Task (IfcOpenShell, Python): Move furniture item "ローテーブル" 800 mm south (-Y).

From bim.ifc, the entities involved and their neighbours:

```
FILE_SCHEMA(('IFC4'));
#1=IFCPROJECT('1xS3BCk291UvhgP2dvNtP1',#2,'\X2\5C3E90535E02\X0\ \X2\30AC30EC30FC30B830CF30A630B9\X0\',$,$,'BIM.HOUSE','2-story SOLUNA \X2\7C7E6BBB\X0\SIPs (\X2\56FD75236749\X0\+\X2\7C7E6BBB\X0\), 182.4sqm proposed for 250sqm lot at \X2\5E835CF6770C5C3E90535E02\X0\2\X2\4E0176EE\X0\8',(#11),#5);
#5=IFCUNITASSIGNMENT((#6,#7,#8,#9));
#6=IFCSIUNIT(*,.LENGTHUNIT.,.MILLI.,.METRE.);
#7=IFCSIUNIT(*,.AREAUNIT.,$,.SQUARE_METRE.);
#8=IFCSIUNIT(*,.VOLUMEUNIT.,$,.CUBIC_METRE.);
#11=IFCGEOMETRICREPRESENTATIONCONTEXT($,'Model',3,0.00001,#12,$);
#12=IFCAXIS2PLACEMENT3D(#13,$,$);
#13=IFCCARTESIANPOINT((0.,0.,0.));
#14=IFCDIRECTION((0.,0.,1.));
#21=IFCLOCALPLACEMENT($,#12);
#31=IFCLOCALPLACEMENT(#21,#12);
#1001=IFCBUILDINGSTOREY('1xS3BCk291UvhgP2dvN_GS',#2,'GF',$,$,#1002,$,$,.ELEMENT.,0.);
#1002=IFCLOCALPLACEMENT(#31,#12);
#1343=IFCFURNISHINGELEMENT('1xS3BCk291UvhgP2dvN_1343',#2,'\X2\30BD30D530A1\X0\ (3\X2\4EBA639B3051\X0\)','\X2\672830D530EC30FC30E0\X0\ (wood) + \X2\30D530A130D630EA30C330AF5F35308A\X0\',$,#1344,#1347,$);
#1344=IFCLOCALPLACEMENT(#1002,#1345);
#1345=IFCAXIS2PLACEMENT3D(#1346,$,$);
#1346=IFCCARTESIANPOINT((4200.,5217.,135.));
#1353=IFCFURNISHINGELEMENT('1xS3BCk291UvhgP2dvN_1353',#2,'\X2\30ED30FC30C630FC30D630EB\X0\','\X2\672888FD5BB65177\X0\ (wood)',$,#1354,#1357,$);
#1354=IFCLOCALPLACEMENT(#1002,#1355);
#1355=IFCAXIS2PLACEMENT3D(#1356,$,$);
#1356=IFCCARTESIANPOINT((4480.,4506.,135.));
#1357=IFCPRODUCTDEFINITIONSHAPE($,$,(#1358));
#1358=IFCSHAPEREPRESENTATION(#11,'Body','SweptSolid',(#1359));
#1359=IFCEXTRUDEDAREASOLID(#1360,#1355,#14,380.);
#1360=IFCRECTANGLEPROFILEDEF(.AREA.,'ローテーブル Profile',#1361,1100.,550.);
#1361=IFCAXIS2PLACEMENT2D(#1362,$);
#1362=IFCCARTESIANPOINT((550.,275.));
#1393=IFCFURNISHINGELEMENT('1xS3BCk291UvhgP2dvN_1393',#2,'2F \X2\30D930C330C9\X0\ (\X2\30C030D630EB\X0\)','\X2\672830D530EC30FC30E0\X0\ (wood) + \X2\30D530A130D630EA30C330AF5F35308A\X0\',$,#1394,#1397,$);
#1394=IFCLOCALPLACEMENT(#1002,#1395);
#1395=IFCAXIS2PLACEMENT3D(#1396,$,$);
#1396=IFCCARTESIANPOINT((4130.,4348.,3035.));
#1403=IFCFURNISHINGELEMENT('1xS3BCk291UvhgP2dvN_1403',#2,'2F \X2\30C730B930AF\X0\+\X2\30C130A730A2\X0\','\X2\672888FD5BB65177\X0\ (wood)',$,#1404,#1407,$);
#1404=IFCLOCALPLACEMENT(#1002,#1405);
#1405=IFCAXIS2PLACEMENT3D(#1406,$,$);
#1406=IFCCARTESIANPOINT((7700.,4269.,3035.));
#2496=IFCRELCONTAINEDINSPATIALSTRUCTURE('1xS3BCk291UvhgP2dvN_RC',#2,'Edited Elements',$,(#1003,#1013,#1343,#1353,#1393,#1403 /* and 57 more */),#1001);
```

```python
import ifcopenshell
import ifcopenshell.api.geometry
import ifcopenshell.util.placement

model = ifcopenshell.open("bim.ifc")

item = model.by_id(1353)
matrix = ifcopenshell.util.placement.get_local_placement(item.ObjectPlacement)
matrix[1, 3] -= 800.0
ifcopenshell.api.geometry.edit_object_placement(model, product=item, matrix=matrix, is_si=False)

print(ifcopenshell.util.placement.get_local_placement(item.ObjectPlacement).round(3) + 0.0)

model.write("bim_edited.ifc")
```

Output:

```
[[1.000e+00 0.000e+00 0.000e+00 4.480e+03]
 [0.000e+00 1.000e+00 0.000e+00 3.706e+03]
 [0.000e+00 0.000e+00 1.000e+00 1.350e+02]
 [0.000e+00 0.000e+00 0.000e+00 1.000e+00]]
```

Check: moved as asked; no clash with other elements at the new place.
